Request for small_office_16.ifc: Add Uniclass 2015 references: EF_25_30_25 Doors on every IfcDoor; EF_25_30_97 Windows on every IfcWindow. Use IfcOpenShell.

First a look at what the model holds.

```python
import ifcopenshell

model = ifcopenshell.open("small_office_16.ifc")
print(model.schema)
print("classifications:", [c.Name for c in model.by_type("IfcClassification")])
for ifc_class in ("IfcDoor", "IfcRoof", "IfcStair", "IfcWall", "IfcWindow"):
    print(ifc_class, len(model.by_type(ifc_class)))
```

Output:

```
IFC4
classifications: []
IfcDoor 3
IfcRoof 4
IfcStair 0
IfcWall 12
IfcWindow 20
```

```python
import ifcopenshell
import ifcopenshell.api.classification

model = ifcopenshell.open("small_office_16.ifc")

system = ifcopenshell.api.classification.add_classification(model, classification="Uniclass 2015")

codes = {
    "IfcDoor": ("EF_25_30_25", "Doors"),
    "IfcWindow": ("EF_25_30_97", "Windows"),
}
for ifc_class, (code, name) in codes.items():
    products = model.by_type(ifc_class)
    ifcopenshell.api.classification.add_reference(
        model, products=products, classification=system, identification=code, name=name
    )
    print(code, len(products))

model.write("small_office_16_edited.ifc")
```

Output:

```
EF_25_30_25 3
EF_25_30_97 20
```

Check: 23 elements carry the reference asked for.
